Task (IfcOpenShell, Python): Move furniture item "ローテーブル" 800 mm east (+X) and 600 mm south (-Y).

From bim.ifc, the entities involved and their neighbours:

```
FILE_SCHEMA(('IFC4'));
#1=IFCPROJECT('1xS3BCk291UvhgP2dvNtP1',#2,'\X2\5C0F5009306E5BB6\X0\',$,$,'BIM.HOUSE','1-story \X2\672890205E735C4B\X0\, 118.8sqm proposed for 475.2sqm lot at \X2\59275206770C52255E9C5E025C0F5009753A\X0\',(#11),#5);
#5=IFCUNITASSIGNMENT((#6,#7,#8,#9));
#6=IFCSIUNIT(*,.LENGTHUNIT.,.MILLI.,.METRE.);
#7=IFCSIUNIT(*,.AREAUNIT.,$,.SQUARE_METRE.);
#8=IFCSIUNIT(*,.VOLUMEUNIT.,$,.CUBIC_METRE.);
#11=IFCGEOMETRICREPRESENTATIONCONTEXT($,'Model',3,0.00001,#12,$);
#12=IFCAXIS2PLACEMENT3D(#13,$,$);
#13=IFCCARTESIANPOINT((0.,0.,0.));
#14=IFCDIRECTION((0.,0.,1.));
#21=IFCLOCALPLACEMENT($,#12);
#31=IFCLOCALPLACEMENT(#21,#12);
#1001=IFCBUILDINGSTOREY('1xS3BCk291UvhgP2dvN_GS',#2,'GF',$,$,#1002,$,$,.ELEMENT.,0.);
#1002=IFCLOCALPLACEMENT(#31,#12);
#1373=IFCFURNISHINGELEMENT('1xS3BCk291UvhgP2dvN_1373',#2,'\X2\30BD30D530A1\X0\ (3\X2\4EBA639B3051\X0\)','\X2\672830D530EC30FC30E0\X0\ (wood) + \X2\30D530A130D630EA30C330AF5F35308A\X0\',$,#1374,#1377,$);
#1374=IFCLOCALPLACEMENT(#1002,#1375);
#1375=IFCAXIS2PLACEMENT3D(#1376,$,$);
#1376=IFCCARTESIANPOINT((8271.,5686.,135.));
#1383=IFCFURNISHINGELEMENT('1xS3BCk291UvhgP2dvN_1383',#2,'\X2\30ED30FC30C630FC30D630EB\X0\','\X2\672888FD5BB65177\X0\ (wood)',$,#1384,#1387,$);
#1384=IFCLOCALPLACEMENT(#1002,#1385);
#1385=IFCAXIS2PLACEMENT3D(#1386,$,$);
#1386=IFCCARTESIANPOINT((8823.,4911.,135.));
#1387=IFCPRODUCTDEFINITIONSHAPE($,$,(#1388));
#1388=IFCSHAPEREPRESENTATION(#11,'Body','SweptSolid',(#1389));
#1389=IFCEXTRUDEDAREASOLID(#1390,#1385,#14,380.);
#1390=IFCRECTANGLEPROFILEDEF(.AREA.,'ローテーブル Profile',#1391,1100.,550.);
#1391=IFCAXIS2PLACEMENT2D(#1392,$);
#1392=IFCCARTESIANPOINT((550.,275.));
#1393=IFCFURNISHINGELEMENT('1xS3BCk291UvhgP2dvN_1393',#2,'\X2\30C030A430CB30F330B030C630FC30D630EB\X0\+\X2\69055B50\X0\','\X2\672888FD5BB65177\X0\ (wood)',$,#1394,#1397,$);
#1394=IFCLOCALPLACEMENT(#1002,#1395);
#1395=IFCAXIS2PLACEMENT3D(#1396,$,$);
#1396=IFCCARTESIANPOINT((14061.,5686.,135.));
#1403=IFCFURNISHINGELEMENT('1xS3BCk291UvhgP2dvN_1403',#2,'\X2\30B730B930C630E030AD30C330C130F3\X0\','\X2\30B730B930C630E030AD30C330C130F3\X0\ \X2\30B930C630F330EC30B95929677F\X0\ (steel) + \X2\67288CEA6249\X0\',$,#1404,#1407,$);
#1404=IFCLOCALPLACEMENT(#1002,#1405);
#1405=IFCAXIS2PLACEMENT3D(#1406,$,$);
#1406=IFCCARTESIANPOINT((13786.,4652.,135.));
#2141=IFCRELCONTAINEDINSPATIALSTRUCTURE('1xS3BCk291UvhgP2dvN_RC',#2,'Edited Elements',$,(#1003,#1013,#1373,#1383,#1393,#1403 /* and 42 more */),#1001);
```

```python
import ifcopenshell
import ifcopenshell.api.geometry
import ifcopenshell.util.placement

model = ifcopenshell.open("bim.ifc")

item = model.by_guid("1xS3BCk291UvhgP2dvN_1383")
matrix = ifcopenshell.util.placement.get_local_placement(item.ObjectPlacement)
matrix[0, 3] += 800.0
matrix[1, 3] -= 600.0
ifcopenshell.api.geometry.edit_object_placement(model, product=item, matrix=matrix, is_si=False)

print(ifcopenshell.util.placement.get_local_placement(item.ObjectPlacement).round(3) + 0.0)

model.write("bim_v2.ifc")
```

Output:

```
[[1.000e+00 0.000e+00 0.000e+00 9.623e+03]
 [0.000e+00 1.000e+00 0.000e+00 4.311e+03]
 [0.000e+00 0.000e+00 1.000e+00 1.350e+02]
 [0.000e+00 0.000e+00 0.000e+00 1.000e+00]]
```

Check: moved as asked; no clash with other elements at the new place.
